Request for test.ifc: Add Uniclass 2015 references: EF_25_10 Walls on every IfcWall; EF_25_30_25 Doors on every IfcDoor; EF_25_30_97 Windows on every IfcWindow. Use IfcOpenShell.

First a look at what the model holds.

```python
import ifcopenshell

model = ifcopenshell.open("test.ifc")
print(model.schema)
print("classifications:", [c.Name for c in model.by_type("IfcClassification")])
for ifc_class in ("IfcDoor", "IfcRoof", "IfcStair", "IfcWall", "IfcWindow"):
    print(ifc_class, len(model.by_type(ifc_class)))
```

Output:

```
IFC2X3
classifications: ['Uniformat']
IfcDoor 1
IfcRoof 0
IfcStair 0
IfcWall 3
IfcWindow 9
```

```python
import ifcopenshell
import ifcopenshell.api.classification

model = ifcopenshell.open("test.ifc")

# IFC2X3 requires Source and Edition and has no link from the project to the system.
system = model.create_entity("IfcClassification", Source="NBS", Edition="2015", Name="Uniclass 2015")

codes = {
    "IfcWall": ("EF_25_10", "Walls"),
    "IfcDoor": ("EF_25_30_25", "Doors"),
    "IfcWindow": ("EF_25_30_97", "Windows"),
}
for ifc_class, (code, name) in codes.items():
    products = model.by_type(ifc_class)
    ifcopenshell.api.classification.add_reference(
        model, products=products, classification=system, identification=code, name=name
    )
    print(code, len(products))

model.write("test-out.ifc")
```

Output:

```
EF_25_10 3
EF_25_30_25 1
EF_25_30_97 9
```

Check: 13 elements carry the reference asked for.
